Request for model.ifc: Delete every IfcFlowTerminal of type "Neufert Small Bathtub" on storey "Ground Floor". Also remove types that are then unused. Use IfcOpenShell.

First a look at what the model holds.

```python
import ifcopenshell
import ifcopenshell.util.element

model = ifcopenshell.open("model.ifc")
print(model.schema)
storey = next(s for s in model.by_type("IfcBuildingStorey") if s.Name == "Ground Floor")
terminals = [e for e in ifcopenshell.util.element.get_decomposition(storey) if e.is_a("IfcFlowTerminal")]
seen = {}
for e in terminals:
    element_type = ifcopenshell.util.element.get_type(e)
    name = element_type.Name if element_type not in (None, e) else None
    seen[name] = seen.get(name, 0) + 1
for name, count in sorted(seen.items(), key=str):
    print(count, "x", name)
```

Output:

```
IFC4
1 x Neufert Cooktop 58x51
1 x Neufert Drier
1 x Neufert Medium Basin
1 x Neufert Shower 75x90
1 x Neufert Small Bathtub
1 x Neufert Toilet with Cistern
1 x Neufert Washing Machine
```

```python
import ifcopenshell
import ifcopenshell.api.root
import ifcopenshell.util.element

model = ifcopenshell.open("model.ifc")

storey = next(s for s in model.by_type("IfcBuildingStorey") if s.Name == "Ground Floor")
terminals = [e for e in ifcopenshell.util.element.get_decomposition(storey) if e.is_a("IfcFlowTerminal")]
targets = [e for e in terminals if (t := ifcopenshell.util.element.get_type(e)) not in (None, e) and t.Name == "Neufert Small Bathtub"]
types = {ifcopenshell.util.element.get_type(e) for e in targets} - {None, *targets}

for e in targets:
    ifcopenshell.api.root.remove_product(model, product=e)
print(len(targets), "removed")

unused = [t for t in types if not ifcopenshell.util.element.get_types(t)]
for t in unused:
    ifcopenshell.api.root.remove_product(model, product=t)
print(len(unused), "unused types removed")

model.write("model_edited.ifc")
```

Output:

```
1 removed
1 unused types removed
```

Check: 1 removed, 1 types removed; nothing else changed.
